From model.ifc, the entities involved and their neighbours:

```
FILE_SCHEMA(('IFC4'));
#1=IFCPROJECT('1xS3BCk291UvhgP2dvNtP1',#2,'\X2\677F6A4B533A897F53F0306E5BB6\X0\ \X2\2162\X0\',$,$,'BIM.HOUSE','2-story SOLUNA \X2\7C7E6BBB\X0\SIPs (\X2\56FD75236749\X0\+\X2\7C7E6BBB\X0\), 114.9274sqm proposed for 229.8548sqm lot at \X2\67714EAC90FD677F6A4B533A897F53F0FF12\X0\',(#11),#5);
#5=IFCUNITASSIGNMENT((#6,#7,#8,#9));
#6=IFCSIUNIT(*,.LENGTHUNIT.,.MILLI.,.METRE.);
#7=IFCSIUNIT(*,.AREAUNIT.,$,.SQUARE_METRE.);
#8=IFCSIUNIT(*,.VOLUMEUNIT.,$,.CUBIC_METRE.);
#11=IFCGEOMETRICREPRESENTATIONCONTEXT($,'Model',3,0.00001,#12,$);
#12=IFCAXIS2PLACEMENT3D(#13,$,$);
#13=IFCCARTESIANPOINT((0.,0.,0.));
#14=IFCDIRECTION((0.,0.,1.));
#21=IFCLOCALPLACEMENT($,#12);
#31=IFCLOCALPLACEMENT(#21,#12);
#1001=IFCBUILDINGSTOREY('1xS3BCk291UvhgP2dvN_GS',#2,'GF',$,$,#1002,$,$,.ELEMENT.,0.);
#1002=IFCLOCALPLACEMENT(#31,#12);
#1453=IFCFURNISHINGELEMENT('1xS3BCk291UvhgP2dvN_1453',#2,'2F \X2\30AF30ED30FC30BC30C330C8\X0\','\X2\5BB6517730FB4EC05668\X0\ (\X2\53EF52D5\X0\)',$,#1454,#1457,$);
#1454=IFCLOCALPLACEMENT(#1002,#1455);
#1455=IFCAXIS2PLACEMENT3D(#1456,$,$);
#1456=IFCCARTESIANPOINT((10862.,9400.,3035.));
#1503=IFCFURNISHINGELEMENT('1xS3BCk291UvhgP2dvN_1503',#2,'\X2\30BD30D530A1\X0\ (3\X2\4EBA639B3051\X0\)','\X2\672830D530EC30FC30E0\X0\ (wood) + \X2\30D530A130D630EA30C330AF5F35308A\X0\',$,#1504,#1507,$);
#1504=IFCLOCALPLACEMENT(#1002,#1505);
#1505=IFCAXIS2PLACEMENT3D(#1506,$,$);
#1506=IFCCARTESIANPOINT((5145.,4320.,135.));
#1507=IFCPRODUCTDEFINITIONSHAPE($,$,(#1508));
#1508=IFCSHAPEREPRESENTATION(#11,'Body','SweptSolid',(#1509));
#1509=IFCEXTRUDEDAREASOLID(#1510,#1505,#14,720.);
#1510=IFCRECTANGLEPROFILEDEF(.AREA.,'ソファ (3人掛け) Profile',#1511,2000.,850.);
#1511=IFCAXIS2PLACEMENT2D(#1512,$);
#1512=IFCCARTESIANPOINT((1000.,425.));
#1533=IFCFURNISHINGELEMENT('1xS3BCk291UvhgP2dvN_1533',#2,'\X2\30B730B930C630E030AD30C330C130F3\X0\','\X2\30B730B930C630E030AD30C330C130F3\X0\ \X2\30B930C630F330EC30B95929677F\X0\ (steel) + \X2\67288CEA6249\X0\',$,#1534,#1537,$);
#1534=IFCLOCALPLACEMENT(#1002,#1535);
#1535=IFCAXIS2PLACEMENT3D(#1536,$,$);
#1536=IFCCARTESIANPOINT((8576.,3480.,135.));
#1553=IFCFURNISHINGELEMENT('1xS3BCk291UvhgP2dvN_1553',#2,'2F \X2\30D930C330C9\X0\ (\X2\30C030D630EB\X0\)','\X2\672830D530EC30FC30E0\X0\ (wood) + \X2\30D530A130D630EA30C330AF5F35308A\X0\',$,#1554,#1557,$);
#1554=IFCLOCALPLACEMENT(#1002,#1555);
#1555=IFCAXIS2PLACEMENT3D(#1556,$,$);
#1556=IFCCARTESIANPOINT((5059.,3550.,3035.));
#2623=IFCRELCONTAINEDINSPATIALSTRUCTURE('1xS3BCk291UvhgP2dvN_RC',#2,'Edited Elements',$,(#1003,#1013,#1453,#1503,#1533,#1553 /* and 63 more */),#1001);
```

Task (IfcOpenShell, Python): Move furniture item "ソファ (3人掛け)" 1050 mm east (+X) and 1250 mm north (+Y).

```python
import ifcopenshell
import ifcopenshell.api.geometry
import ifcopenshell.util.placement
import ifcopenshell.util.unit

model = ifcopenshell.open("model.ifc")
unit_scale = ifcopenshell.util.unit.calculate_unit_scale(model)

item = model.by_guid("1xS3BCk291UvhgP2dvN_1503")
matrix = ifcopenshell.util.placement.get_local_placement(item.ObjectPlacement)
matrix[0, 3] += 1.05 / unit_scale
matrix[1, 3] += 1.25 / unit_scale
ifcopenshell.api.geometry.edit_object_placement(model, product=item, matrix=matrix, is_si=False)

print(ifcopenshell.util.placement.get_local_placement(item.ObjectPlacement).round(3) + 0.0)

model.write("model-out.ifc")
```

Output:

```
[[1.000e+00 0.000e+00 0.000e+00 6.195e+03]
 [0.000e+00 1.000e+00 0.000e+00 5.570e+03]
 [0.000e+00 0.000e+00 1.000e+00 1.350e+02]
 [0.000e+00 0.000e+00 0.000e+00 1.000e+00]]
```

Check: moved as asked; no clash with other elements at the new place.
